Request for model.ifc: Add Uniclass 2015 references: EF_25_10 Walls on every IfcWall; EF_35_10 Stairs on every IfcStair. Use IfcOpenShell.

First a look at what the model holds.

```python
import ifcopenshell

model = ifcopenshell.open("model.ifc")
print(model.schema)
print("classifications:", [c.Name for c in model.by_type("IfcClassification")])
for ifc_class in ("IfcDoor", "IfcRoof", "IfcStair", "IfcWall", "IfcWindow"):
    print(ifc_class, len(model.by_type(ifc_class)))
```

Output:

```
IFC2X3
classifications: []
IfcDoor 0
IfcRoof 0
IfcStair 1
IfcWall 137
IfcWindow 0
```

```python
import ifcopenshell
import ifcopenshell.api.classification

model = ifcopenshell.open("model.ifc")

# IFC2X3 requires Source and Edition and has no link from the project to the system.
system = model.create_entity("IfcClassification", Source="NBS", Edition="2015", Name="Uniclass 2015")

codes = {
    "IfcWall": ("EF_25_10", "Walls"),
    "IfcStair": ("EF_35_10", "Stairs"),
}
for ifc_class, (code, name) in codes.items():
    products = model.by_type(ifc_class)
    ifcopenshell.api.classification.add_reference(
        model, products=products, classification=system, identification=code, name=name
    )
    print(code, len(products))

model.write("model_updated.ifc")
```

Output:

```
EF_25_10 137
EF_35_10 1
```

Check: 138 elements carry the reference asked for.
